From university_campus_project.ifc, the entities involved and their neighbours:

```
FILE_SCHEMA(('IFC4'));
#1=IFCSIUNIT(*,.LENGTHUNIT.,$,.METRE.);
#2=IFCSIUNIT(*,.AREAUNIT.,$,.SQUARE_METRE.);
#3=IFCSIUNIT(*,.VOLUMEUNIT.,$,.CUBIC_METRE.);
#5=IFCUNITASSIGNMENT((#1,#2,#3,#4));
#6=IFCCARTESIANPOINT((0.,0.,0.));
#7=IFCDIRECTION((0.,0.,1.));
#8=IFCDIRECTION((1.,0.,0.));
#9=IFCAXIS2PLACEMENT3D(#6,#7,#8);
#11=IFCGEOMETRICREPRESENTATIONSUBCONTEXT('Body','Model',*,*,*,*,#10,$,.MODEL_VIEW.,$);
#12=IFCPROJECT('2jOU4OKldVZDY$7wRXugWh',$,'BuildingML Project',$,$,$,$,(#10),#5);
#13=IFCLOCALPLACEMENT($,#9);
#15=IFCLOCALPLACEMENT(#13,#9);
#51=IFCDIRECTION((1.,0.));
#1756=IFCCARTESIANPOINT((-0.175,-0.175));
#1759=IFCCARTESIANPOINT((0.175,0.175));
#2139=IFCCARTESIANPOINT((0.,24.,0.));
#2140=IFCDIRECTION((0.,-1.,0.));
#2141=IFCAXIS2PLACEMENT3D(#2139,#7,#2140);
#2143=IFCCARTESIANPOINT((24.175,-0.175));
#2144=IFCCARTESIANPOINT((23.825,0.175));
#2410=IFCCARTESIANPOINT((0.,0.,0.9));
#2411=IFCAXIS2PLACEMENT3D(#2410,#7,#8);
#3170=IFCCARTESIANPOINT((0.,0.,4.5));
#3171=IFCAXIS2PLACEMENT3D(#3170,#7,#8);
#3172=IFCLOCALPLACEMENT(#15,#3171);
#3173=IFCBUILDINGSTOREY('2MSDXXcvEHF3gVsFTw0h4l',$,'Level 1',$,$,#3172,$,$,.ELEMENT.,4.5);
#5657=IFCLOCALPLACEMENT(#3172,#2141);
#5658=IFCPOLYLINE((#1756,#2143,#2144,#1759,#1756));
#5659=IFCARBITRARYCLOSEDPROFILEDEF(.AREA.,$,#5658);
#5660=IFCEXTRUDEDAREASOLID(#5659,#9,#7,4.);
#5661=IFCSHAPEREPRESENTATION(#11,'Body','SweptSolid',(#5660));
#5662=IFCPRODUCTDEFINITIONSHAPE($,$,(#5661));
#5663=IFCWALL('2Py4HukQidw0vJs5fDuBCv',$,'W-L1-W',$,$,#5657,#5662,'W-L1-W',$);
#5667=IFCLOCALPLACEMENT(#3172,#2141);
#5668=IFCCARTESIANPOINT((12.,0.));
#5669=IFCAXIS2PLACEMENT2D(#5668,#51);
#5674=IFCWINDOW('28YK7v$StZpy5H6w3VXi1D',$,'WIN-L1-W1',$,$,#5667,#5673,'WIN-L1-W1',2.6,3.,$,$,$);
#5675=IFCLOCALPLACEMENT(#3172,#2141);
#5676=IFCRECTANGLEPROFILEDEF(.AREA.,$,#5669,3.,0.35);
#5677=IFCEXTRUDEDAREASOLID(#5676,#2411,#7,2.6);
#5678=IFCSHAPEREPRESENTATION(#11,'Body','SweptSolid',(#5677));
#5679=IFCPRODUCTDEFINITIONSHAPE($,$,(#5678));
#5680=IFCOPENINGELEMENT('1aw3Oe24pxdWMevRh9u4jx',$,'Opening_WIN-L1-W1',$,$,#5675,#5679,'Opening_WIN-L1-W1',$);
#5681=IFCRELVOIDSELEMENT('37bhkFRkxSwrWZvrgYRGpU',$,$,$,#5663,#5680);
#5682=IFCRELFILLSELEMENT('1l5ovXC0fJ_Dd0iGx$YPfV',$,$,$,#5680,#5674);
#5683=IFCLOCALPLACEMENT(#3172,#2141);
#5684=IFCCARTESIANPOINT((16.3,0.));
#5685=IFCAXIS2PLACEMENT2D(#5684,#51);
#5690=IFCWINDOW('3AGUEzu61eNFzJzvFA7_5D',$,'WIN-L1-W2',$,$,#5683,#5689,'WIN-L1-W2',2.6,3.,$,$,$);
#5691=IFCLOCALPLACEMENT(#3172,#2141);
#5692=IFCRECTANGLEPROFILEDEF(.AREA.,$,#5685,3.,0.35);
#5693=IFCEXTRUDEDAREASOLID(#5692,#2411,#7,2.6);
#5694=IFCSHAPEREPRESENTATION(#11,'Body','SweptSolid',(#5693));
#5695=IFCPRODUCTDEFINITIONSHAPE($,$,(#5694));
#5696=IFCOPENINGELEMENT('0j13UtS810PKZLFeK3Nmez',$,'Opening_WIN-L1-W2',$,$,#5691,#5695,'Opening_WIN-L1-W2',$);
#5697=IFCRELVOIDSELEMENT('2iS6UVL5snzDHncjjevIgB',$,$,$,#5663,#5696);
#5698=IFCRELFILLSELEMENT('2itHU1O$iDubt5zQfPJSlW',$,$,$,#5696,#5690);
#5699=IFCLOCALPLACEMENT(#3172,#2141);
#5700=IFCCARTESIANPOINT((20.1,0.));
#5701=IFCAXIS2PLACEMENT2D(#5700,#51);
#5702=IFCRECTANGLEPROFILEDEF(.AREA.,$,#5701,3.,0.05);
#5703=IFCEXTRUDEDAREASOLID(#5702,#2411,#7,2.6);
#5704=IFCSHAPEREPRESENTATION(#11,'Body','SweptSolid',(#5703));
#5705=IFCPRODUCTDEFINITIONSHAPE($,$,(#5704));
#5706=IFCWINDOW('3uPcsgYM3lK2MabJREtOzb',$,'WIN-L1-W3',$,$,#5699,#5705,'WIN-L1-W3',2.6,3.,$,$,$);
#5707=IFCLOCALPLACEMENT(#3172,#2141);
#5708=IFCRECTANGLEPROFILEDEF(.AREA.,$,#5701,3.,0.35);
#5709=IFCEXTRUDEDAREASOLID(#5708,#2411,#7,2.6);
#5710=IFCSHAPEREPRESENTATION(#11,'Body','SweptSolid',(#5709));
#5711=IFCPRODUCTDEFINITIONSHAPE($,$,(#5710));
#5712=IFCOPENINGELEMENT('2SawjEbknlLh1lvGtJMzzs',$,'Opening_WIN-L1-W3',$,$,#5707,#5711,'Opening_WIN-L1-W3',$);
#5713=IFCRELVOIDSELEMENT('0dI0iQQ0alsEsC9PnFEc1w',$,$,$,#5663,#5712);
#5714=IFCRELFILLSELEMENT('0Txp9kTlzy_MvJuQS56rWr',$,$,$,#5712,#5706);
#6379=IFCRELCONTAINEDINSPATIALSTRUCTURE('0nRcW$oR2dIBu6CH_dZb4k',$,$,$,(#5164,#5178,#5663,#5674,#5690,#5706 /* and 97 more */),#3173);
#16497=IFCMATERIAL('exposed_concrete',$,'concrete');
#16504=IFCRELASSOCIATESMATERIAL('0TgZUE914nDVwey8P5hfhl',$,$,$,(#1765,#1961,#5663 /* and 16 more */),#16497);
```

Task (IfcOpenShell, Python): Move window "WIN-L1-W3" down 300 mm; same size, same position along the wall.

```python
import numpy as np
import ifcopenshell
import ifcopenshell.api.geometry
import ifcopenshell.util.placement
import ifcopenshell.util.unit

model = ifcopenshell.open("university_campus_project.ifc")
unit_scale = ifcopenshell.util.unit.calculate_unit_scale(model)

window = model.by_guid("3uPcsgYM3lK2MabJREtOzb")
opening = window.FillsVoids[0].RelatingOpeningElement
dz = -0.3

shift = np.array([0.0, 0.0, dz])
# The window is not placed relative to its opening, so move both.
for product in (opening, window):
    matrix = ifcopenshell.util.placement.get_local_placement(product.ObjectPlacement)
    matrix[:3, 3] += shift
    ifcopenshell.api.geometry.edit_object_placement(model, product=product, matrix=matrix, is_si=False)

print(f"moved by {dz * unit_scale:+.3f} m")

model.write("university_campus_project_updated.ifc")
```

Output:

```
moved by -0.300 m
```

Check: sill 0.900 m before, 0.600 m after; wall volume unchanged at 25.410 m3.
